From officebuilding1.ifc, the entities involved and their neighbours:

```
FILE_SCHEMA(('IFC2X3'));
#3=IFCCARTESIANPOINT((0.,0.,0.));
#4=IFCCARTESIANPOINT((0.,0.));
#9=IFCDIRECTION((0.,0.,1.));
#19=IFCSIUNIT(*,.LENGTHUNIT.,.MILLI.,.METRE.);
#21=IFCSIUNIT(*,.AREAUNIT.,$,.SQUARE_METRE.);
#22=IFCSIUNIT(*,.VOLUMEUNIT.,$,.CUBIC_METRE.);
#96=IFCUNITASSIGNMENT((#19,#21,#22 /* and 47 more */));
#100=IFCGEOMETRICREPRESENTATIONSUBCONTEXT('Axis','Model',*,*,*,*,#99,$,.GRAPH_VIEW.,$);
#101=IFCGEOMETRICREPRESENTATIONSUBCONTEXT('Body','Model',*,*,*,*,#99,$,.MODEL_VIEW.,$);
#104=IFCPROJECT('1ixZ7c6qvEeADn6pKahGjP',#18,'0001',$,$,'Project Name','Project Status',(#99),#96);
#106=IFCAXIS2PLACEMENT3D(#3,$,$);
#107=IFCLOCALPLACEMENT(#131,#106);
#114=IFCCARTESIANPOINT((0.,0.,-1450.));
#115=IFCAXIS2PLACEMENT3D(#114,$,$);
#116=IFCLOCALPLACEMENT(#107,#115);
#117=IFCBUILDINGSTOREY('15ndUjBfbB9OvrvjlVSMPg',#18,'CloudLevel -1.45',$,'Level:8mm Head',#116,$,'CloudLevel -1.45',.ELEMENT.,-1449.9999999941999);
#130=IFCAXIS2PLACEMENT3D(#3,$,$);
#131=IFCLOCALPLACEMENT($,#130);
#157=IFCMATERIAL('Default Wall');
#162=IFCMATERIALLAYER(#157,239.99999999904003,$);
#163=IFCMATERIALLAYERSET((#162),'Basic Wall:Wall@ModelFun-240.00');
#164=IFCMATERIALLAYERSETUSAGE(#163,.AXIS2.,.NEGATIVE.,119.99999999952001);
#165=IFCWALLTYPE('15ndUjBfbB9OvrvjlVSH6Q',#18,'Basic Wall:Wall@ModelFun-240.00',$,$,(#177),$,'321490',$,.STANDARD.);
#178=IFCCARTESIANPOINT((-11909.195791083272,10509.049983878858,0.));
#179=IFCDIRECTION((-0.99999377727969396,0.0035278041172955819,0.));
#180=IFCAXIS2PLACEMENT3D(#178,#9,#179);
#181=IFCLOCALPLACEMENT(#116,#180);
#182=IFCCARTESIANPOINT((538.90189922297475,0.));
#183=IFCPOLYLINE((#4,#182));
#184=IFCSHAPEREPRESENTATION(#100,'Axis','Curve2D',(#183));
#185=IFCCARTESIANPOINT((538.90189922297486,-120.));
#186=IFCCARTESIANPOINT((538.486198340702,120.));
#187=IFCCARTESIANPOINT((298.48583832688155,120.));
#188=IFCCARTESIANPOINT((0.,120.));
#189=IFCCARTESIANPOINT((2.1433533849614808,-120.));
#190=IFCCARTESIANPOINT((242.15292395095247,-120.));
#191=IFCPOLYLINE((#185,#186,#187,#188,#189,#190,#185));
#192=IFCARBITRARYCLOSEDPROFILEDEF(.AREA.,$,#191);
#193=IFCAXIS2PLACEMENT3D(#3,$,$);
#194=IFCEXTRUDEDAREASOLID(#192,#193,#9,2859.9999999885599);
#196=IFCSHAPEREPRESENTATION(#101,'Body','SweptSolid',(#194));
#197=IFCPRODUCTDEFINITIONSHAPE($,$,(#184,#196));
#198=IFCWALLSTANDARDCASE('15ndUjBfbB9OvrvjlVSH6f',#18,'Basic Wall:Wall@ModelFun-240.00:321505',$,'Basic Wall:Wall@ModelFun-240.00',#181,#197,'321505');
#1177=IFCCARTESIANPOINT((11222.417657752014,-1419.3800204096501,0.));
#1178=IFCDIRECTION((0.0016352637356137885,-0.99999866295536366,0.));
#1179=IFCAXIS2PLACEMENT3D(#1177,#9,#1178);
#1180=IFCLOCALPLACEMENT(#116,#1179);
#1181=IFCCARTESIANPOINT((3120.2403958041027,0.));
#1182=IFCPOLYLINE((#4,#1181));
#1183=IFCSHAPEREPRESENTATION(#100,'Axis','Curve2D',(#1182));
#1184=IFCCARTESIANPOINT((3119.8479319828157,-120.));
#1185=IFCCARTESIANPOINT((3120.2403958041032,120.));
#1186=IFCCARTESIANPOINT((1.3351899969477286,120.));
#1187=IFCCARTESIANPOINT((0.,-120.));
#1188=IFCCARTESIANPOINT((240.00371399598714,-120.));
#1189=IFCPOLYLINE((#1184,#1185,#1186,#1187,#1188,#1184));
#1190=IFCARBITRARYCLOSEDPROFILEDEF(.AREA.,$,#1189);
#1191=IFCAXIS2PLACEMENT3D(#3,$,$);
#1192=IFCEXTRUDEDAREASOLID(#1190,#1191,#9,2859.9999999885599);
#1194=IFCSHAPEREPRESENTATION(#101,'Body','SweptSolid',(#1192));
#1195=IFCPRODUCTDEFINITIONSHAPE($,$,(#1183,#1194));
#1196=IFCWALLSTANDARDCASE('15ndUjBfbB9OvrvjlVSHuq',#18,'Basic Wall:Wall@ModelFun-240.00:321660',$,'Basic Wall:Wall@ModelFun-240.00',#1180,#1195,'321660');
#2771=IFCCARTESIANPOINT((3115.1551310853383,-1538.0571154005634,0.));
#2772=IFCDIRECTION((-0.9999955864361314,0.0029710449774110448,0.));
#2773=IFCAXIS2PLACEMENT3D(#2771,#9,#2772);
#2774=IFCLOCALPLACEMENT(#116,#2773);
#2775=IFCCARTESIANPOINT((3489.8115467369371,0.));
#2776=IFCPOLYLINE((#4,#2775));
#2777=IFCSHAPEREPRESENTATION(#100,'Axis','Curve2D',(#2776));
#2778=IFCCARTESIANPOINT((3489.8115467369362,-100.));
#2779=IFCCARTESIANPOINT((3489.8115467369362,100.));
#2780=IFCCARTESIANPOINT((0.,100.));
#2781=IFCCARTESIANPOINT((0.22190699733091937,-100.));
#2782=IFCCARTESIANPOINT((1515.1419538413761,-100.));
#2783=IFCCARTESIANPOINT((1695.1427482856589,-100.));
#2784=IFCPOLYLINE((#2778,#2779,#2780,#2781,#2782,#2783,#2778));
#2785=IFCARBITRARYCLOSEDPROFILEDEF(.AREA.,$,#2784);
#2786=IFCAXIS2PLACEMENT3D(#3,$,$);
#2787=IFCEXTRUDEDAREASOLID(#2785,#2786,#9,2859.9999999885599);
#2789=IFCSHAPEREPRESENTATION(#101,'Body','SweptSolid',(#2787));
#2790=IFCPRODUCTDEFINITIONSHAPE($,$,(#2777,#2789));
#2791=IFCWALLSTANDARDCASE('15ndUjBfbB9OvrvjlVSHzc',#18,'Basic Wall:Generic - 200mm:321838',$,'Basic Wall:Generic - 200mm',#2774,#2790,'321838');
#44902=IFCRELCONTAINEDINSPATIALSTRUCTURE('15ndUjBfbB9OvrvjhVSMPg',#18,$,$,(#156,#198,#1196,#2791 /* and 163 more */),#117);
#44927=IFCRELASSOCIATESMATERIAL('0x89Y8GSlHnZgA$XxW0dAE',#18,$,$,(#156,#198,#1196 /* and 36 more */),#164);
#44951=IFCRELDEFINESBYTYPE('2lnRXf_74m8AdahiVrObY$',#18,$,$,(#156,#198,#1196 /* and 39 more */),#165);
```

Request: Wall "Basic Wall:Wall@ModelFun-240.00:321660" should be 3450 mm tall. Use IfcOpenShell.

```python
import ifcopenshell
import ifcopenshell.geom
import ifcopenshell.util.representation
import ifcopenshell.util.shape
import ifcopenshell.util.unit

model = ifcopenshell.open("officebuilding1.ifc")
unit_scale = ifcopenshell.util.unit.calculate_unit_scale(model)
settings = ifcopenshell.geom.settings()


def volume(element):
    """Net volume in cubic metres, openings subtracted."""
    shape = ifcopenshell.geom.create_shape(settings, element)
    return ifcopenshell.util.shape.get_volume(shape.geometry)


wall = model.by_guid("15ndUjBfbB9OvrvjlVSHuq")
before = volume(wall)

body = ifcopenshell.util.representation.get_representation(wall, "Model", "Body")
solid = body.Items[0]
old_height = solid.Depth
solid.Depth = 3.45 / unit_scale
after = volume(wall)

print(f"height {old_height:g} -> {solid.Depth:g}, volume {before:.3f} -> {after:.3f} m3")

model.write("officebuilding1_rev.ifc")
```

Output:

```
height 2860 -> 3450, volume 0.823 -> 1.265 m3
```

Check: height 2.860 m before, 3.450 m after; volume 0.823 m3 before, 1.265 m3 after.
